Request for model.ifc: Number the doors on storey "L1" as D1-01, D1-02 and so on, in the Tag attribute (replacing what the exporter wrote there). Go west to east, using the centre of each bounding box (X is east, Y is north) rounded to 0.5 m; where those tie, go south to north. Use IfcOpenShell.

First a look at what the model holds.

```python
import ifcopenshell
import ifcopenshell.util.element
import ifcopenshell.util.placement

model = ifcopenshell.open("model.ifc")
print(model.schema)
storey = next(s for s in model.by_type("IfcBuildingStorey") if s.Name == "L1")
doors = [e for e in ifcopenshell.util.element.get_decomposition(storey) if e.is_a("IfcDoor")]
for e in sorted(doors, key=lambda e: e.id()):
    origin = ifcopenshell.util.placement.get_local_placement(e.ObjectPlacement)[:3, 3]
    print(e.id(), e.Tag, e.Name, origin.round(2) + 0.0, sep=" | ")
```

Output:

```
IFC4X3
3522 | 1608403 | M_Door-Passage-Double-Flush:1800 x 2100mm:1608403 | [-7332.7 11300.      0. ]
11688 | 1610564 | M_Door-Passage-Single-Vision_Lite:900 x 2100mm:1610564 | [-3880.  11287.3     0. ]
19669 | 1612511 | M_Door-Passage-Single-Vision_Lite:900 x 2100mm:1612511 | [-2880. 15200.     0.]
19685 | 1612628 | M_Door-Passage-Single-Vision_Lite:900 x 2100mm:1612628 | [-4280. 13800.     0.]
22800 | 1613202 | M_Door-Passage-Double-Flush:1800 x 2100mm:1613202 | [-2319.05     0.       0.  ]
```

```python
import ifcopenshell
import ifcopenshell.geom
import ifcopenshell.util.element
import ifcopenshell.util.shape

model = ifcopenshell.open("model.ifc")
settings = ifcopenshell.geom.settings()
settings.set("use-world-coords", True)


def centre(element):
    shape = ifcopenshell.geom.create_shape(settings, element)
    return ifcopenshell.util.shape.get_bbox_centroid(shape.geometry)


storey = next(s for s in model.by_type("IfcBuildingStorey") if s.Name == "L1")
doors = [e for e in ifcopenshell.util.element.get_decomposition(storey) if e.is_a("IfcDoor")]

# Insertion points can sit at a corner or the storey origin, so sort by the geometry (in metres).
centres = {e: centre(e) for e in doors}
doors.sort(key=lambda e: (round(centres[e][0] / 0.5), centres[e][1]))

for i, e in enumerate(doors, start=1):
    number = f"D1-{i:02d}"
    e.Tag = number
    print(e.id(), number)

model.write("model-out.ifc")
```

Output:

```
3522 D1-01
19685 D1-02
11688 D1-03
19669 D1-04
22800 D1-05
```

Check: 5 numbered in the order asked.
